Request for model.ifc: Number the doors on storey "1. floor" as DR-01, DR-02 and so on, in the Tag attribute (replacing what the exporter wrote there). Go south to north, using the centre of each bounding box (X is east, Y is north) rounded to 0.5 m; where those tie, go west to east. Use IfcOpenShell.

First a look at what the model holds.

```python
import ifcopenshell
import ifcopenshell.util.element
import ifcopenshell.util.placement

model = ifcopenshell.open("model.ifc")
print(model.schema)
storey = next(s for s in model.by_type("IfcBuildingStorey") if s.Name == "1. floor")
doors = [e for e in ifcopenshell.util.element.get_decomposition(storey) if e.is_a("IfcDoor")]
for e in sorted(doors, key=lambda e: e.id()):
    origin = ifcopenshell.util.placement.get_local_placement(e.ObjectPlacement)[:3, 3]
    print(e.id(), e.Tag, e.Name, origin.round(2) + 0.0, sep=" | ")
```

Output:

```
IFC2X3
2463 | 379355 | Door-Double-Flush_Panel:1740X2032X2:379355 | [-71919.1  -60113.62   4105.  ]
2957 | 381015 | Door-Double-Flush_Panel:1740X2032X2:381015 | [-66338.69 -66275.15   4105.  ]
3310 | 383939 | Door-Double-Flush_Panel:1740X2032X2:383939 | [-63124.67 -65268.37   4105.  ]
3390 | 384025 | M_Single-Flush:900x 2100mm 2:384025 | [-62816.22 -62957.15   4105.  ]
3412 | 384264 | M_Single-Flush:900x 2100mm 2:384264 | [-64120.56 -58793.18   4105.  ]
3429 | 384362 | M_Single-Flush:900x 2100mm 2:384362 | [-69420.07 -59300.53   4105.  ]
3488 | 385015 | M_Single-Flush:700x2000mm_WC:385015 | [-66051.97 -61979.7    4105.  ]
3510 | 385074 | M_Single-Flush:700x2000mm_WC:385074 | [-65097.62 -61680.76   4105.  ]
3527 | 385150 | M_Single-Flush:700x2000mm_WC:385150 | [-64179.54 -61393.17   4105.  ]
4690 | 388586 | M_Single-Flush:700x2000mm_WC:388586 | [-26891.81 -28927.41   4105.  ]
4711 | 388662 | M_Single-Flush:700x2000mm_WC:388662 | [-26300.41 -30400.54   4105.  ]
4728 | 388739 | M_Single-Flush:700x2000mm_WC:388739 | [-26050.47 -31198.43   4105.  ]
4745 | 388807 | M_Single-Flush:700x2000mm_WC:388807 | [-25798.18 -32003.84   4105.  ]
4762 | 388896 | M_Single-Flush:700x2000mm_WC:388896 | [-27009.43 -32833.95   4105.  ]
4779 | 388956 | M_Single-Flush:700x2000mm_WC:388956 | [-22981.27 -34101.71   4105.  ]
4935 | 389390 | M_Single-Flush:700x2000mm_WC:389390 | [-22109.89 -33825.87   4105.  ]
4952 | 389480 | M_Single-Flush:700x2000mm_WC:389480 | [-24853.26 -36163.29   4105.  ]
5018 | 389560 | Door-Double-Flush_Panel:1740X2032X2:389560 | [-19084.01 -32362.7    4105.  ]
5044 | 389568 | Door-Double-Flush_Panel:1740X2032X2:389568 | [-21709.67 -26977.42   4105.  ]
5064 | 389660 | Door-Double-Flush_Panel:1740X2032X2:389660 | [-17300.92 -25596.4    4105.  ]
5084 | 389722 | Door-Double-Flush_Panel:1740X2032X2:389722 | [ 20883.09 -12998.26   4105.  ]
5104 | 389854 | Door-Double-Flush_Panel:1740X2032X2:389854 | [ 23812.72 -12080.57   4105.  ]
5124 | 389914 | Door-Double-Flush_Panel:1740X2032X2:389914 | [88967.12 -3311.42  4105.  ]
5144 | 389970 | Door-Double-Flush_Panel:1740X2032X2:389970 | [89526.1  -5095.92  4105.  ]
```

```python
import ifcopenshell
import ifcopenshell.geom
import ifcopenshell.util.element
import ifcopenshell.util.shape

model = ifcopenshell.open("model.ifc")
settings = ifcopenshell.geom.settings()
settings.set("use-world-coords", True)


def centre(element):
    shape = ifcopenshell.geom.create_shape(settings, element)
    return ifcopenshell.util.shape.get_bbox_centroid(shape.geometry)


storey = next(s for s in model.by_type("IfcBuildingStorey") if s.Name == "1. floor")
doors = [e for e in ifcopenshell.util.element.get_decomposition(storey) if e.is_a("IfcDoor")]

# Insertion points can sit at a corner or the storey origin, so sort by the geometry (in metres).
centres = {e: centre(e) for e in doors}
doors.sort(key=lambda e: (round(centres[e][1] / 0.5), centres[e][0]))

for i, e in enumerate(doors, start=1):
    number = f"DR-{i:02d}"
    e.Tag = number
    print(e.id(), number)

model.write("model-out.ifc")
```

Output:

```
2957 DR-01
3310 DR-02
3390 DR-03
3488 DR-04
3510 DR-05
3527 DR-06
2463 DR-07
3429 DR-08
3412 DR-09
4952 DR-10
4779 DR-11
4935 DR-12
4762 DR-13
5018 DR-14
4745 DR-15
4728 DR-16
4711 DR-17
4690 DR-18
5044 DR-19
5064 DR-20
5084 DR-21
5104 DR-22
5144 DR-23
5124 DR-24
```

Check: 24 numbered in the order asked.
